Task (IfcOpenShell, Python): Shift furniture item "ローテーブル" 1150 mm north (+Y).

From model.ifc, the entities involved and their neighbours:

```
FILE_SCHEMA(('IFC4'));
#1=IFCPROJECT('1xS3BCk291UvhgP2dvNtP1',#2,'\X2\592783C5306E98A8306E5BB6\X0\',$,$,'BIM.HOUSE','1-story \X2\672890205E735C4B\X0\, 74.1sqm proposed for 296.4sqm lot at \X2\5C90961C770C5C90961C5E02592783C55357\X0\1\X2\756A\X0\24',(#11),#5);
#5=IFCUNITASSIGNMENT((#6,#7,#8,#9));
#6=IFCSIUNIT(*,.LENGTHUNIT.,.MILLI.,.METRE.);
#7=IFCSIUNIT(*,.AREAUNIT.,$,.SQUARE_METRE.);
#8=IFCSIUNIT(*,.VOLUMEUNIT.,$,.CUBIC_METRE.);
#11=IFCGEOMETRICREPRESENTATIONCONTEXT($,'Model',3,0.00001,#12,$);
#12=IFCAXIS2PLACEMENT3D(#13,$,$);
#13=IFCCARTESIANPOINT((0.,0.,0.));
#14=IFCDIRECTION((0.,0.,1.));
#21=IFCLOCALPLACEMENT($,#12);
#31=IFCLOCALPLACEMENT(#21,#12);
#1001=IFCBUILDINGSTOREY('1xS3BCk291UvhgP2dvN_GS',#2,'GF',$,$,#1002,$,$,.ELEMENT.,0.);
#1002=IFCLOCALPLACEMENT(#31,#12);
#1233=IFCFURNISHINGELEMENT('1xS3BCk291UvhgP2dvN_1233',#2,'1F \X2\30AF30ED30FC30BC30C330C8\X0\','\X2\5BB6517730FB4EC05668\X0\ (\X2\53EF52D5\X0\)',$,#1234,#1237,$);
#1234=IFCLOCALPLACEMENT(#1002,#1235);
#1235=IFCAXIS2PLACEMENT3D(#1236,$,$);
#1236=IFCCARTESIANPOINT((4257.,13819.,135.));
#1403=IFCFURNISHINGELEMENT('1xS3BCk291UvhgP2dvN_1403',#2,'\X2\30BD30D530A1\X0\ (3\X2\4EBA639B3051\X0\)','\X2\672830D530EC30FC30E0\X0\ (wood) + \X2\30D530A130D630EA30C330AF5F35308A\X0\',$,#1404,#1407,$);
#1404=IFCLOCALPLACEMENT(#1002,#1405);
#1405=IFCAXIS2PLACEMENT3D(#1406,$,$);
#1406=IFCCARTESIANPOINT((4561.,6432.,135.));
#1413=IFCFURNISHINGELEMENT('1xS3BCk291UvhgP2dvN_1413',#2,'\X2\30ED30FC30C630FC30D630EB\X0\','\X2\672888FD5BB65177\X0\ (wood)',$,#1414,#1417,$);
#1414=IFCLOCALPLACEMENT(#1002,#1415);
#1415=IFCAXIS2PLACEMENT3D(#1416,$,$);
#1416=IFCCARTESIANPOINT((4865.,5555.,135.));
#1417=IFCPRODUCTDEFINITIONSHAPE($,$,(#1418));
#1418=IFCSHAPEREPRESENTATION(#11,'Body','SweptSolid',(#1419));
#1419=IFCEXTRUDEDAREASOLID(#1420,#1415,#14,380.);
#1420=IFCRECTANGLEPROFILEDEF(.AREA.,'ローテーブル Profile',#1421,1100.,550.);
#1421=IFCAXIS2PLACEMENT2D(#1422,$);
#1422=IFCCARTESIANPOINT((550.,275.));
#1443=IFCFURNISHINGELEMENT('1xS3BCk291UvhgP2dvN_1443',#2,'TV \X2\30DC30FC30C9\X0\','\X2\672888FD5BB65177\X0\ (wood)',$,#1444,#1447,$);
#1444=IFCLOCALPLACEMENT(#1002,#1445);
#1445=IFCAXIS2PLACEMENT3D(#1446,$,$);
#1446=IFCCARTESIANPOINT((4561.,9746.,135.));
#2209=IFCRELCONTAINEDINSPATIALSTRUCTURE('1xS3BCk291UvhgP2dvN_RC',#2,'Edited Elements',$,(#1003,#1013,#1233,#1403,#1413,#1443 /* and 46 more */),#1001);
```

```python
import ifcopenshell
import ifcopenshell.api.geometry
import ifcopenshell.util.placement
import ifcopenshell.util.unit

model = ifcopenshell.open("model.ifc")
unit_scale = ifcopenshell.util.unit.calculate_unit_scale(model)

item = model.by_id(1413)
matrix = ifcopenshell.util.placement.get_local_placement(item.ObjectPlacement)
matrix[1, 3] += 1.15 / unit_scale
ifcopenshell.api.geometry.edit_object_placement(model, product=item, matrix=matrix, is_si=False)

print(ifcopenshell.util.placement.get_local_placement(item.ObjectPlacement).round(3) + 0.0)

model.write("model_edited.ifc")
```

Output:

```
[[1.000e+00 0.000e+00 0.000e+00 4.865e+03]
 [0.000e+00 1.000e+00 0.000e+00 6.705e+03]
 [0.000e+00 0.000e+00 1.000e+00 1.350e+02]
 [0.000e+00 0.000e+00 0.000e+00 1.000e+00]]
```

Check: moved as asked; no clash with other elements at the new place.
